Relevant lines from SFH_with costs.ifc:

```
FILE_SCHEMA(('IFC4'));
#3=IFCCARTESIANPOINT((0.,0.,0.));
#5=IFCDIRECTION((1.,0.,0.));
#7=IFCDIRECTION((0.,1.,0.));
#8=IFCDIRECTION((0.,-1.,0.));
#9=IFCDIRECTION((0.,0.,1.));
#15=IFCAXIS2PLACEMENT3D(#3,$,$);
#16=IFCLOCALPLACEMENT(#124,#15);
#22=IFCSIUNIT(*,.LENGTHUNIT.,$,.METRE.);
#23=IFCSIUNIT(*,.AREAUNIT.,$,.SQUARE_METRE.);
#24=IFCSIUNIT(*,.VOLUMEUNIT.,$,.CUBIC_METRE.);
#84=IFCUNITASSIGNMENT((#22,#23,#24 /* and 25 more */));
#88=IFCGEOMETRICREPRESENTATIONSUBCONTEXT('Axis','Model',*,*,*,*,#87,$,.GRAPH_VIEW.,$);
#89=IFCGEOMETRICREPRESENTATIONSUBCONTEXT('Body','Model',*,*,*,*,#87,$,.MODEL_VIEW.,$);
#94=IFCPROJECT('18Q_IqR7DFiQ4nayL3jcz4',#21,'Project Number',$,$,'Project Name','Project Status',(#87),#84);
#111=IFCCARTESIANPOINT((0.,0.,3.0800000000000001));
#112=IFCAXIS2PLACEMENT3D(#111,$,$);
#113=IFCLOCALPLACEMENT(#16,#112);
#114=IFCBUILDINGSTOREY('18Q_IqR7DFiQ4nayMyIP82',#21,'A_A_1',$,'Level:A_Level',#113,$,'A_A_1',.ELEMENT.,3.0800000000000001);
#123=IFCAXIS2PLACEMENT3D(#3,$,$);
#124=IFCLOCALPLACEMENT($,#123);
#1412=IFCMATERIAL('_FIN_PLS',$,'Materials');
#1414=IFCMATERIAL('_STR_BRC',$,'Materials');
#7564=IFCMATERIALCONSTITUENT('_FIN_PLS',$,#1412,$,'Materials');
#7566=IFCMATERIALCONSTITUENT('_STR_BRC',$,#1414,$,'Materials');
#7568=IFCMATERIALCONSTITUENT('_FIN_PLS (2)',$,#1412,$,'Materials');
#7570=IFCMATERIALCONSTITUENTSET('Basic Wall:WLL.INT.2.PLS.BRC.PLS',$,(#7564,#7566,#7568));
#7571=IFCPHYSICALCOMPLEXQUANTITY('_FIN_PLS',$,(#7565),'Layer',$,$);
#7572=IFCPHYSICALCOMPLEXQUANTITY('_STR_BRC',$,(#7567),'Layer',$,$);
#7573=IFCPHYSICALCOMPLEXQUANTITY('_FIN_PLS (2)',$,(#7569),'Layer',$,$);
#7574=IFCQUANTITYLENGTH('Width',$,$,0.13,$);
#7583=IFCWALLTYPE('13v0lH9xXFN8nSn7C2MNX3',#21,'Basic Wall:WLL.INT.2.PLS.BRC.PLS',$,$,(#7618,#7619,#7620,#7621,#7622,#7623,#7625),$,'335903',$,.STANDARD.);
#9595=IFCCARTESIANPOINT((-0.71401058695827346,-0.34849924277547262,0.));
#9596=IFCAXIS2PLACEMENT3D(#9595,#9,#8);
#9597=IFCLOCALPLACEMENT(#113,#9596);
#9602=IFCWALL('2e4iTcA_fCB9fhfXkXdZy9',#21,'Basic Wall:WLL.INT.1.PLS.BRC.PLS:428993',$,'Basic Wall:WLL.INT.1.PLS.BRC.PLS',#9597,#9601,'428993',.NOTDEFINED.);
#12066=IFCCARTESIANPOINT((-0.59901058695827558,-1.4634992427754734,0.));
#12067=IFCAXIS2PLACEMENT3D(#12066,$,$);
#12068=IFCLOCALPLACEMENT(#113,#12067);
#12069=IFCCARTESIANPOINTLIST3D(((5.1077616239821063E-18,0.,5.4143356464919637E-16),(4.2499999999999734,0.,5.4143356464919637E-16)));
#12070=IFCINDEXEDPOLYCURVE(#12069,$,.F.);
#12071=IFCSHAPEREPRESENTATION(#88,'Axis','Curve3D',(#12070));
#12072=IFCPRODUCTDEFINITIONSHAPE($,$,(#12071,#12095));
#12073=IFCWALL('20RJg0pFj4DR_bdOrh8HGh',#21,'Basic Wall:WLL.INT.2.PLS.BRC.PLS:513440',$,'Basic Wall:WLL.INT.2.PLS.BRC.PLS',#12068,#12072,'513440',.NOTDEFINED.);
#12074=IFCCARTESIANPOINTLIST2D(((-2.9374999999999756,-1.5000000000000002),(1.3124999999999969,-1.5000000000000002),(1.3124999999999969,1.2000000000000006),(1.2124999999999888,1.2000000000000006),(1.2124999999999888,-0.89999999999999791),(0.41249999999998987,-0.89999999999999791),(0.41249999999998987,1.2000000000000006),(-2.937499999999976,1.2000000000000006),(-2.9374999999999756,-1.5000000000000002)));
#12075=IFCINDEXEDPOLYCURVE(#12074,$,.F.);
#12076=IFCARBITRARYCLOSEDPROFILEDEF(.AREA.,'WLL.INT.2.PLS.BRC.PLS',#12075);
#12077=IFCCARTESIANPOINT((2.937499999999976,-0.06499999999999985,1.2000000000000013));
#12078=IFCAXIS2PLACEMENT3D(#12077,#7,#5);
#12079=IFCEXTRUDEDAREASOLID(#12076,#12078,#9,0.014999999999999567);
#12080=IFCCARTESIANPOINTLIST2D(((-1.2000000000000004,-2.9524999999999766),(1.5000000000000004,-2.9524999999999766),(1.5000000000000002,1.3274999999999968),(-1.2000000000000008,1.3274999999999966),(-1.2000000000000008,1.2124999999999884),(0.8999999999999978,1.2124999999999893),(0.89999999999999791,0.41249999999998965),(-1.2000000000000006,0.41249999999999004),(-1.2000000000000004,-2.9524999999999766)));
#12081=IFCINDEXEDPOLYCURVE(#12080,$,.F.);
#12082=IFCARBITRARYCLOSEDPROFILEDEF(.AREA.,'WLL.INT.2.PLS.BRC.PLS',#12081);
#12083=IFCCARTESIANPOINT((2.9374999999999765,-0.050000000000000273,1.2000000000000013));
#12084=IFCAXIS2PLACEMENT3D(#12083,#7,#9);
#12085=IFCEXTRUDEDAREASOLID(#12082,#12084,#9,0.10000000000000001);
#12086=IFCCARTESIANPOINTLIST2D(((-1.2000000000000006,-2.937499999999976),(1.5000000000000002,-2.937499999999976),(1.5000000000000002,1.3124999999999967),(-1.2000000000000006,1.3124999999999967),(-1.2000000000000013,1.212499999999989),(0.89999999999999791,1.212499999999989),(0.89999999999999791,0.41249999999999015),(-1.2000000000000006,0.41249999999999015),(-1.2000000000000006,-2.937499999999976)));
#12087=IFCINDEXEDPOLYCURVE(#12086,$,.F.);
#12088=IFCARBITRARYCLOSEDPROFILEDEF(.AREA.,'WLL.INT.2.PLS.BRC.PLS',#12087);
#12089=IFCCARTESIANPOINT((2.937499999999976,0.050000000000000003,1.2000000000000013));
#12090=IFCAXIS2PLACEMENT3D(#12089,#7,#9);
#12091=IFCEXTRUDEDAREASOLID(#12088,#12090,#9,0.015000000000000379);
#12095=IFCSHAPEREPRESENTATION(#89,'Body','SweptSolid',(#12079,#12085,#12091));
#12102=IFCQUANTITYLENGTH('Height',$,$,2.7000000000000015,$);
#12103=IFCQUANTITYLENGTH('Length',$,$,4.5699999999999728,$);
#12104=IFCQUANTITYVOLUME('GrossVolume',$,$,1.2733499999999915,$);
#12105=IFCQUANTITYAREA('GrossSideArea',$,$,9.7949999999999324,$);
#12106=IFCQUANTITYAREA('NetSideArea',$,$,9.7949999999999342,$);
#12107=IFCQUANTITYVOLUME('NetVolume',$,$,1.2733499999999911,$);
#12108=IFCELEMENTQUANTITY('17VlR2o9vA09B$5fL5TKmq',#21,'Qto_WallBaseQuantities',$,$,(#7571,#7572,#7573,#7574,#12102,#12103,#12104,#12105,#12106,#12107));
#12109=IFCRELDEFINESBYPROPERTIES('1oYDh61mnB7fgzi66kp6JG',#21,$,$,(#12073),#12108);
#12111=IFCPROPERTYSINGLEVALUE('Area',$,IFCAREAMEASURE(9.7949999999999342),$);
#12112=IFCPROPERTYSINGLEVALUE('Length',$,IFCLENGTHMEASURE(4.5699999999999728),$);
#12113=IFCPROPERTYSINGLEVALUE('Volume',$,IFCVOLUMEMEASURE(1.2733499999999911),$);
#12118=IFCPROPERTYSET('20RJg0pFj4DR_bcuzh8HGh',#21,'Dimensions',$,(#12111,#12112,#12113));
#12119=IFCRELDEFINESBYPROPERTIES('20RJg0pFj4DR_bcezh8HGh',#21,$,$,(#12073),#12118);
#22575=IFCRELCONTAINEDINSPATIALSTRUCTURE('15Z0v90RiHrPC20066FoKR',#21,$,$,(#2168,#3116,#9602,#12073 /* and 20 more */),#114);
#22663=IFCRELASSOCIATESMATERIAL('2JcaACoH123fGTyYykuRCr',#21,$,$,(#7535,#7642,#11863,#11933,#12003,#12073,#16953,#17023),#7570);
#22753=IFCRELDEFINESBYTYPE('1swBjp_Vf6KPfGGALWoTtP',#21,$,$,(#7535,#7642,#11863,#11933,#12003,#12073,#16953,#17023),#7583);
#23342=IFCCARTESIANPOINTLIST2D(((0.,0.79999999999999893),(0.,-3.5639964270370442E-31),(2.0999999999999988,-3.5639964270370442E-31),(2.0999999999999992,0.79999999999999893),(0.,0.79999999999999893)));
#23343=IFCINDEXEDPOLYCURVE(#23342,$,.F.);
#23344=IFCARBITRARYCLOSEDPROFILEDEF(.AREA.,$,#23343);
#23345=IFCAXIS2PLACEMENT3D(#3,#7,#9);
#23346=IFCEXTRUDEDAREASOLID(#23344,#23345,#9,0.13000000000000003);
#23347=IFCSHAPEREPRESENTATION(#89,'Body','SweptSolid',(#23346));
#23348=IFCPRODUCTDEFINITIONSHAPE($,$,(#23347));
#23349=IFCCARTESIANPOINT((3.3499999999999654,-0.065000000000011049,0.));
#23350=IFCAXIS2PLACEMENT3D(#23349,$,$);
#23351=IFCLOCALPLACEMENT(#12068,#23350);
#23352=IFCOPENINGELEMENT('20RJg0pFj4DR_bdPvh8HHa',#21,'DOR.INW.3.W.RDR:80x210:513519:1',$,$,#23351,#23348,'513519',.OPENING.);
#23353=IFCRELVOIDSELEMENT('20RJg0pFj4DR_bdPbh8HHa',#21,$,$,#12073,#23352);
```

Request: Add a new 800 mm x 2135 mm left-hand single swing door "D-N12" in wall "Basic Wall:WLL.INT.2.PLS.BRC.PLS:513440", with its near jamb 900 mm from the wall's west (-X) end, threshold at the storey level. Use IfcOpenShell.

```python
import numpy as np
import ifcopenshell
import ifcopenshell.api.feature
import ifcopenshell.api.geometry
import ifcopenshell.api.pset
import ifcopenshell.api.root
import ifcopenshell.api.spatial
import ifcopenshell.geom
import ifcopenshell.util.element
import ifcopenshell.util.placement
import ifcopenshell.util.representation
import ifcopenshell.util.shape
import ifcopenshell.util.unit

model = ifcopenshell.open("SFH_with costs.ifc")
unit_scale = ifcopenshell.util.unit.calculate_unit_scale(model)
area_scale = ifcopenshell.util.unit.calculate_unit_scale(model, "AREAUNIT")
volume_scale = ifcopenshell.util.unit.calculate_unit_scale(model, "VOLUMEUNIT")
settings = ifcopenshell.geom.settings()


def volume(element):
    """Net volume in cubic metres, openings subtracted."""
    shape = ifcopenshell.geom.create_shape(settings, element)
    return ifcopenshell.util.shape.get_volume(shape.geometry)


wall = model.by_guid("20RJg0pFj4DR_bdOrh8HGh")
storey = ifcopenshell.util.element.get_container(wall, ifc_class="IfcBuildingStorey")
context = ifcopenshell.util.representation.get_context(model, "Model", "Body", "MODEL_VIEW")
before = volume(wall)

width, height, from_end, sill = 0.8, 2.135, 0.9, 0.0  # metres

# The wall runs along its own X axis, and the end named is its -X end.
wall_shape = ifcopenshell.geom.create_shape(settings, wall)
x, y, z = ifcopenshell.util.shape.get_vertices(wall_shape.geometry).T
start = x.min() + from_end
face, thickness = float(y.min()), float(y.max() - y.min())
wall_matrix = ifcopenshell.util.placement.get_local_placement(wall.ObjectPlacement)
level = ifcopenshell.util.placement.get_local_placement(storey.ObjectPlacement)[2, 3]


def in_wall(x, y):
    """Placement at x, y metres in the wall's axes, at sill height."""
    matrix = wall_matrix.copy()
    matrix[:, 3] = wall_matrix @ np.array([x / unit_scale, y / unit_scale, 0.0, 1.0])
    matrix[2, 3] = level + sill / unit_scale
    return matrix


# Opening: a box that overshoots both wall faces by 50 mm.
opening = ifcopenshell.api.root.create_entity(model, ifc_class="IfcOpeningElement", predefined_type="OPENING")
box = ifcopenshell.api.geometry.add_wall_representation(
    model, context=context, length=width, height=height, thickness=thickness + 0.1
)
ifcopenshell.api.geometry.assign_representation(model, product=opening, representation=box)
ifcopenshell.api.geometry.edit_object_placement(model, product=opening, matrix=in_wall(start, face - 0.05), is_si=False)
ifcopenshell.api.feature.add_feature(model, feature=opening, element=wall)

door = ifcopenshell.api.root.create_entity(model, ifc_class="IfcDoor", name="D-N12", predefined_type="DOOR")
door.OverallWidth, door.OverallHeight = width / unit_scale, height / unit_scale
door.OperationType = "SINGLE_SWING_LEFT"
body = ifcopenshell.api.geometry.add_door_representation(
    model,
    context=context,
    overall_width=door.OverallWidth,
    overall_height=door.OverallHeight,
    operation_type="SINGLE_SWING_LEFT",
    lining_properties={"LiningDepth": thickness / unit_scale, "ThresholdDepth": thickness / unit_scale},
)
ifcopenshell.api.geometry.assign_representation(model, product=door, representation=body)
ifcopenshell.api.spatial.assign_container(model, products=[door], relating_structure=storey)
ifcopenshell.api.feature.add_filling(model, opening=opening, element=door)

# The lining spans the wall, so the door starts at the wall face.
ifcopenshell.api.geometry.edit_object_placement(model, product=door, matrix=in_wall(start, face), is_si=False)

after = volume(wall)

# Update the wall's stored quantities.
qto = model.by_id(ifcopenshell.util.element.get_pset(wall, "Qto_WallBaseQuantities", should_inherit=False)["id"])
ifcopenshell.api.pset.edit_qto(model, qto=qto, properties={
    "NetSideArea": after / thickness / area_scale,
    "NetVolume": after / volume_scale,
})
pset = model.by_id(ifcopenshell.util.element.get_pset(wall, "Dimensions", should_inherit=False)["id"])
ifcopenshell.api.pset.edit_pset(model, pset=pset, properties={
    "Area": model.create_entity("IfcAreaMeasure", after / thickness / area_scale),
    "Volume": model.create_entity("IfcVolumeMeasure", after / volume_scale),
})

print(f"wall volume {before:.3f} -> {after:.3f} m3")

model.write("SFH_with costs-out.ifc")
```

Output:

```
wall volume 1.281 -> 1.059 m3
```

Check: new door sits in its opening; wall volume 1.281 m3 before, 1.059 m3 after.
